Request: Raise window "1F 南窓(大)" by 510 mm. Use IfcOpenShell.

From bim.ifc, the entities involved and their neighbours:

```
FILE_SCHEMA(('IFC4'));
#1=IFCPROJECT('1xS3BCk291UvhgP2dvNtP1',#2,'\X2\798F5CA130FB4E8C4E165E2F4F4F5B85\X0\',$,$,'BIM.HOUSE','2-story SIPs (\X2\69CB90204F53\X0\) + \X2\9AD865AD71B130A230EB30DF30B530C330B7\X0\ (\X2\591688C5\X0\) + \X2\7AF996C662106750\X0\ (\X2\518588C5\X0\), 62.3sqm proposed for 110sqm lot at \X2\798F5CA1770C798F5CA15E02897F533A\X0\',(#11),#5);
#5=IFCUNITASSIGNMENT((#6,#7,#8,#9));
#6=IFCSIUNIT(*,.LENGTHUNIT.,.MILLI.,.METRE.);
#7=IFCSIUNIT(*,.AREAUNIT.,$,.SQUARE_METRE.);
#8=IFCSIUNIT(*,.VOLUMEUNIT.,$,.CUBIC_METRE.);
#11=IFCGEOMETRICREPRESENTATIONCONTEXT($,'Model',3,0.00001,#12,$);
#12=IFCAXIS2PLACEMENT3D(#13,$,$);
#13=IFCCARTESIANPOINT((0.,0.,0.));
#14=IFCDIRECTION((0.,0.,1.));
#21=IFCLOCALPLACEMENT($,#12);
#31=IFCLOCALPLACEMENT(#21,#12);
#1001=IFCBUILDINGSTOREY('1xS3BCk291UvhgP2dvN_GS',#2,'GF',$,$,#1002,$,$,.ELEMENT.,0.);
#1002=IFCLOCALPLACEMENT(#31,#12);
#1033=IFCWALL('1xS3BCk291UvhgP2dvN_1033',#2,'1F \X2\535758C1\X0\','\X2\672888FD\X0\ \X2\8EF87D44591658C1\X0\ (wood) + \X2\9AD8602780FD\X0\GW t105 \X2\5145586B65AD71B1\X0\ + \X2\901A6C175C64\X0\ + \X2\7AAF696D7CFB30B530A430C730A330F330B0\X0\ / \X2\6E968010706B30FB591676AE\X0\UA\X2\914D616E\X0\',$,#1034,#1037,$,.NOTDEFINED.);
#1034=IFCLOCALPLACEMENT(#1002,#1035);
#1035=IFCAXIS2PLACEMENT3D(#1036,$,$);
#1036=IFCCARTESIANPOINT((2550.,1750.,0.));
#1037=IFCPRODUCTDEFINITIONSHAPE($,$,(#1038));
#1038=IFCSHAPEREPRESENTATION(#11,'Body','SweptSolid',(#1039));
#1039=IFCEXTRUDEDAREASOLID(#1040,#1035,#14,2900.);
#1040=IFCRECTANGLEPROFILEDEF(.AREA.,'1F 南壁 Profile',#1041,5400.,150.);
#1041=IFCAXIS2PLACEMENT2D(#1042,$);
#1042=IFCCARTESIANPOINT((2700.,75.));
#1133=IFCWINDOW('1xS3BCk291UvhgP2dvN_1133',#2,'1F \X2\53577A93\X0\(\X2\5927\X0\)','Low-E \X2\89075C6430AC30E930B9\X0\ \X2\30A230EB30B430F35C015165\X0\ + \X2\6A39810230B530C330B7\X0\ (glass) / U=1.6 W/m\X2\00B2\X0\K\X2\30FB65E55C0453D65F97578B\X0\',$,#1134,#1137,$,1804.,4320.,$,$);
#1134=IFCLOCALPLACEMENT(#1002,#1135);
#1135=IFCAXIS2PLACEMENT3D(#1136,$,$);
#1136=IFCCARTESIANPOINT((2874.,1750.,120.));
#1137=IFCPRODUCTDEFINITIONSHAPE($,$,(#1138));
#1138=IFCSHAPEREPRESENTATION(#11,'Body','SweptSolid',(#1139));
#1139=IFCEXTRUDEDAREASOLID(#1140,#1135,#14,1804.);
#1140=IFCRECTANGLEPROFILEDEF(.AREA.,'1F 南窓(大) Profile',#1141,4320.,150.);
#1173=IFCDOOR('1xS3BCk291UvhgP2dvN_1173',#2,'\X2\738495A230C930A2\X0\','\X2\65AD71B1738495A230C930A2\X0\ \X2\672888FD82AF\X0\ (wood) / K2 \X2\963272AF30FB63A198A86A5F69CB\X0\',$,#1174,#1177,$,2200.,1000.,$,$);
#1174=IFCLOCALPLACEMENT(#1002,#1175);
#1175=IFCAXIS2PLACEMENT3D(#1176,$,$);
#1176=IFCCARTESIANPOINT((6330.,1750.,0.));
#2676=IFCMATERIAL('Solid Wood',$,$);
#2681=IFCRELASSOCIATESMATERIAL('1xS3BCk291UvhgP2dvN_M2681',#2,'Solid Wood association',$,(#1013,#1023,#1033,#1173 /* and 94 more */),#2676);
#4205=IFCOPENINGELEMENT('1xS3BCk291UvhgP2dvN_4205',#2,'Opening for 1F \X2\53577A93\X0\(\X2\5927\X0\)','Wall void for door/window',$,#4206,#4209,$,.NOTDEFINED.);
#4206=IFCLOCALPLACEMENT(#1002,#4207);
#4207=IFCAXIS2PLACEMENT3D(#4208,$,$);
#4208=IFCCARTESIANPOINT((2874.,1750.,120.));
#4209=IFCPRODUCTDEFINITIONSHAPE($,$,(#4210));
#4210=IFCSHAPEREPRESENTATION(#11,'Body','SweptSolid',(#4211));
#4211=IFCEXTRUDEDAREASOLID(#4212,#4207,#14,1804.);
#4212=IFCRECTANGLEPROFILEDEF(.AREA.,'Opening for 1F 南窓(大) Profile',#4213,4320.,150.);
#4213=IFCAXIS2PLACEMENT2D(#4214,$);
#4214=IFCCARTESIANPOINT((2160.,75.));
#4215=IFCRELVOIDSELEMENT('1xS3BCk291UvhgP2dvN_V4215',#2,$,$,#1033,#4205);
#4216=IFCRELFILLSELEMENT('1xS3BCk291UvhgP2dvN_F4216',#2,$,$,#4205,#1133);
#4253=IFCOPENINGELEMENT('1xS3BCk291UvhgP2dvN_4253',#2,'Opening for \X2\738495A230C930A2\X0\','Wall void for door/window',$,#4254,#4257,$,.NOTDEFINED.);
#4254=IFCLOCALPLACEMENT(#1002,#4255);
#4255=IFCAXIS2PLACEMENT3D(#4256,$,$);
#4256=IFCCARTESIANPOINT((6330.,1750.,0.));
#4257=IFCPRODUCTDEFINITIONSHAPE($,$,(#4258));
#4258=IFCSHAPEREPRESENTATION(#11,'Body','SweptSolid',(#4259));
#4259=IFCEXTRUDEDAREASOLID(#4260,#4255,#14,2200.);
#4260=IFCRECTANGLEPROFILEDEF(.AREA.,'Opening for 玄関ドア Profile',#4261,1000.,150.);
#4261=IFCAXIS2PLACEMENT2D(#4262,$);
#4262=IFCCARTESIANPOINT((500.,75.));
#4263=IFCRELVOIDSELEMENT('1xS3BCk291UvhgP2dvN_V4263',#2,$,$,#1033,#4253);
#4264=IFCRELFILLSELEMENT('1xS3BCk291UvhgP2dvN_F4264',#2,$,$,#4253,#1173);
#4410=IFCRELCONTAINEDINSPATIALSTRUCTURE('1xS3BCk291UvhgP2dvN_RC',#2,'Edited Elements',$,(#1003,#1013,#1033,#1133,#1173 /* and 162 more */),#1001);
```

```python
import numpy as np
import ifcopenshell
import ifcopenshell.api.geometry
import ifcopenshell.util.placement
import ifcopenshell.util.unit

model = ifcopenshell.open("bim.ifc")
unit_scale = ifcopenshell.util.unit.calculate_unit_scale(model)

window = model.by_id(1133)
opening = window.FillsVoids[0].RelatingOpeningElement
dz = 0.51 / unit_scale

shift = np.array([0.0, 0.0, dz])
# The window is not placed relative to its opening, so move both.
for product in (opening, window):
    matrix = ifcopenshell.util.placement.get_local_placement(product.ObjectPlacement)
    matrix[:3, 3] += shift
    ifcopenshell.api.geometry.edit_object_placement(model, product=product, matrix=matrix, is_si=False)

print(f"moved by {dz * unit_scale:+.3f} m")

model.write("bim_edited.ifc")
```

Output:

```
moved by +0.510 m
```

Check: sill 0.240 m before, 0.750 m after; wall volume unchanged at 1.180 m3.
